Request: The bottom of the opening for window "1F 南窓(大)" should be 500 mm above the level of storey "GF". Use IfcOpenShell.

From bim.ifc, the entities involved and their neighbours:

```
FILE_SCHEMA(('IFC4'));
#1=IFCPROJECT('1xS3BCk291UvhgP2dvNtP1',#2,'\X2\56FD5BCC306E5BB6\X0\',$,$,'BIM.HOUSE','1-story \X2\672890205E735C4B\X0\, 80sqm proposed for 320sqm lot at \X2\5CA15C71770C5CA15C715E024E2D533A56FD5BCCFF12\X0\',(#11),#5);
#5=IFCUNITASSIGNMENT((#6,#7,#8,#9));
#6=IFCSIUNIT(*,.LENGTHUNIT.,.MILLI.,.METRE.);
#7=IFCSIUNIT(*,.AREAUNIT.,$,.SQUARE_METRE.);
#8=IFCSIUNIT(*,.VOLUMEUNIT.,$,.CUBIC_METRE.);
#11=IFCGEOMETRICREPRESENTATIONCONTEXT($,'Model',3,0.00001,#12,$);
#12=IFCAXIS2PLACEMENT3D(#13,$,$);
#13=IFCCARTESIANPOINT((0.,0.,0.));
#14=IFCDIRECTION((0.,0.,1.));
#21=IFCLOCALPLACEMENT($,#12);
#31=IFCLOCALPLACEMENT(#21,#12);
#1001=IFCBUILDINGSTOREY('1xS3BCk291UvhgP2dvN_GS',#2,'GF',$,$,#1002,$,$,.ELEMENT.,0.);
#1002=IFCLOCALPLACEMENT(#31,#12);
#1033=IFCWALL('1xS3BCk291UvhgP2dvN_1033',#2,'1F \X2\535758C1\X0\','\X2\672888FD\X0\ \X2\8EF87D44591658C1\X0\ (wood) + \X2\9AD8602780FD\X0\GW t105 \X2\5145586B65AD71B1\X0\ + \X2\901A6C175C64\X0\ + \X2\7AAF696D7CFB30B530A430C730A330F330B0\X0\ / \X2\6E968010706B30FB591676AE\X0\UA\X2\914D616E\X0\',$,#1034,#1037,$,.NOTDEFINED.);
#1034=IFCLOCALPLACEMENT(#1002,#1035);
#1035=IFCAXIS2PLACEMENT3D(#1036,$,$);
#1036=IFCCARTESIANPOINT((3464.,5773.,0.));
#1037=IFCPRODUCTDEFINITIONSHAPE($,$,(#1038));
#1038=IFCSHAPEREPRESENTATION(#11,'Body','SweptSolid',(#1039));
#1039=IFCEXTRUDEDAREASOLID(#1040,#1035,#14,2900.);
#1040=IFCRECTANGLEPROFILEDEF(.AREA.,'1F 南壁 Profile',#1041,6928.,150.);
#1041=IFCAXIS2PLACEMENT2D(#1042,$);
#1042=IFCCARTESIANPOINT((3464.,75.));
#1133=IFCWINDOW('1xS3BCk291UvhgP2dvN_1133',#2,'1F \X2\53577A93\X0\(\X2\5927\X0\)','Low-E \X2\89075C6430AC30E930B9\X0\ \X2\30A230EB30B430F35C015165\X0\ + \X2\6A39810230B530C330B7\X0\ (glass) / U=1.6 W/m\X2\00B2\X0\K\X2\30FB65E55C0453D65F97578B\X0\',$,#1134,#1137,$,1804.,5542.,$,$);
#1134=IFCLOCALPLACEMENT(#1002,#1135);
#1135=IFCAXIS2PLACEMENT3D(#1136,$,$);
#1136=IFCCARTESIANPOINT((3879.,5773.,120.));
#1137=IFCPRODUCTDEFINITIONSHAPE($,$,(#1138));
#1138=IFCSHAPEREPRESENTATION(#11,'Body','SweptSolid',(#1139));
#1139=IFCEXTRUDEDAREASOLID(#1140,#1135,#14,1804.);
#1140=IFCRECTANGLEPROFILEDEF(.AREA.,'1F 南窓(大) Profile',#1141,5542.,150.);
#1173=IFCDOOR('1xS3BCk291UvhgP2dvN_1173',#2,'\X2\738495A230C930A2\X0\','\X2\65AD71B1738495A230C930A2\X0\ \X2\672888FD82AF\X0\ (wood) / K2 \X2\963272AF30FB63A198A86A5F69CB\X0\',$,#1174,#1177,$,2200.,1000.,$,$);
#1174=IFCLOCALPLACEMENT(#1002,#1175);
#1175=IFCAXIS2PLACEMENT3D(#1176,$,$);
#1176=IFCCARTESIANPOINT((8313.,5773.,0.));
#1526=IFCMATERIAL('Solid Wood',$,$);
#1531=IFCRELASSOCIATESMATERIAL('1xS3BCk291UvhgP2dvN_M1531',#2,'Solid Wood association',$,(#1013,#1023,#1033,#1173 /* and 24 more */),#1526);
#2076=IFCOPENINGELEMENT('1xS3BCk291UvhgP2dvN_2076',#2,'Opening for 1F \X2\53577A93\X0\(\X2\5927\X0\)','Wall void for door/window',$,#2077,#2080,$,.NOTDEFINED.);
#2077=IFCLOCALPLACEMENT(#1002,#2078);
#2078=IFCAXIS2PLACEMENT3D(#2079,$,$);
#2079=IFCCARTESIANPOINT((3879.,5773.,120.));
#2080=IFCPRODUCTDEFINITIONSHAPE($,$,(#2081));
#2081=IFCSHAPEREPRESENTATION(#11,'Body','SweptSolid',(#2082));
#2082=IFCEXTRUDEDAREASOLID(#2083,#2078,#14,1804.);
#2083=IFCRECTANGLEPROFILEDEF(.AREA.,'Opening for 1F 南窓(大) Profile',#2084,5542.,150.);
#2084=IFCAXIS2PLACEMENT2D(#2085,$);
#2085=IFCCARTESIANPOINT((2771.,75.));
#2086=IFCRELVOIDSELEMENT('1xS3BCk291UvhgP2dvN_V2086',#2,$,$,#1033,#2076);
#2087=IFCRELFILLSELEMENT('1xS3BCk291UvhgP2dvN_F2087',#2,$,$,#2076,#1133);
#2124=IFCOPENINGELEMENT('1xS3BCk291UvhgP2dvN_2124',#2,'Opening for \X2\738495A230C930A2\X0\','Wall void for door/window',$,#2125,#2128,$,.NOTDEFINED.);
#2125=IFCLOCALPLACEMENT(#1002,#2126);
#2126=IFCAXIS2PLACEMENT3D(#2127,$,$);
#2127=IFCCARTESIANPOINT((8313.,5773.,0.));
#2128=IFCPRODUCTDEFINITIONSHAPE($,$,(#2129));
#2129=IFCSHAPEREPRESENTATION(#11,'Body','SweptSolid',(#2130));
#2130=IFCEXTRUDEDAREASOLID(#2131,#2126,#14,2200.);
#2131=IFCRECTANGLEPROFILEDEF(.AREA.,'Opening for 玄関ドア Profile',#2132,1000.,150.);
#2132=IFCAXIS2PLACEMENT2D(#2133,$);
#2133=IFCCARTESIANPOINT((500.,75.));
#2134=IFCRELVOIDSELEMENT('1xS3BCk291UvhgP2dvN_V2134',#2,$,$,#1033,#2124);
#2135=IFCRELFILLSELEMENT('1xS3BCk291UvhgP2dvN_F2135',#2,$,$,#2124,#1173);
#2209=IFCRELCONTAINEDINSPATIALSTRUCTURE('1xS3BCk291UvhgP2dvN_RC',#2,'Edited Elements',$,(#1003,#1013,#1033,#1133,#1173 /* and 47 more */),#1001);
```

```python
import numpy as np
import ifcopenshell
import ifcopenshell.api.geometry
import ifcopenshell.geom
import ifcopenshell.util.element
import ifcopenshell.util.placement
import ifcopenshell.util.shape
import ifcopenshell.util.unit

model = ifcopenshell.open("bim.ifc")
unit_scale = ifcopenshell.util.unit.calculate_unit_scale(model)

window = model.by_guid("1xS3BCk291UvhgP2dvN_1133")
opening = window.FillsVoids[0].RelatingOpeningElement
storey = ifcopenshell.util.element.get_container(window, ifc_class="IfcBuildingStorey")
level = ifcopenshell.util.placement.get_local_placement(storey.ObjectPlacement)[2, 3]

# The opening's origin need not be at the sill, so measure its lowest point.
shape = ifcopenshell.geom.create_shape(ifcopenshell.geom.settings(), opening)
bottom = ifcopenshell.util.shape.get_shape_bottom_elevation(shape, shape.geometry) / unit_scale
dz = level + 500.0 - bottom

shift = np.array([0.0, 0.0, dz])
# The window is not placed relative to its opening, so move both.
for product in (opening, window):
    matrix = ifcopenshell.util.placement.get_local_placement(product.ObjectPlacement)
    matrix[:3, 3] += shift
    ifcopenshell.api.geometry.edit_object_placement(model, product=product, matrix=matrix, is_si=False)

print(f"moved by {dz * unit_scale:+.3f} m")

model.write("bim_edited.ifc")
```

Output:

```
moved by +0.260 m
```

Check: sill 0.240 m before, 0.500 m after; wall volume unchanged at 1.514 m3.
